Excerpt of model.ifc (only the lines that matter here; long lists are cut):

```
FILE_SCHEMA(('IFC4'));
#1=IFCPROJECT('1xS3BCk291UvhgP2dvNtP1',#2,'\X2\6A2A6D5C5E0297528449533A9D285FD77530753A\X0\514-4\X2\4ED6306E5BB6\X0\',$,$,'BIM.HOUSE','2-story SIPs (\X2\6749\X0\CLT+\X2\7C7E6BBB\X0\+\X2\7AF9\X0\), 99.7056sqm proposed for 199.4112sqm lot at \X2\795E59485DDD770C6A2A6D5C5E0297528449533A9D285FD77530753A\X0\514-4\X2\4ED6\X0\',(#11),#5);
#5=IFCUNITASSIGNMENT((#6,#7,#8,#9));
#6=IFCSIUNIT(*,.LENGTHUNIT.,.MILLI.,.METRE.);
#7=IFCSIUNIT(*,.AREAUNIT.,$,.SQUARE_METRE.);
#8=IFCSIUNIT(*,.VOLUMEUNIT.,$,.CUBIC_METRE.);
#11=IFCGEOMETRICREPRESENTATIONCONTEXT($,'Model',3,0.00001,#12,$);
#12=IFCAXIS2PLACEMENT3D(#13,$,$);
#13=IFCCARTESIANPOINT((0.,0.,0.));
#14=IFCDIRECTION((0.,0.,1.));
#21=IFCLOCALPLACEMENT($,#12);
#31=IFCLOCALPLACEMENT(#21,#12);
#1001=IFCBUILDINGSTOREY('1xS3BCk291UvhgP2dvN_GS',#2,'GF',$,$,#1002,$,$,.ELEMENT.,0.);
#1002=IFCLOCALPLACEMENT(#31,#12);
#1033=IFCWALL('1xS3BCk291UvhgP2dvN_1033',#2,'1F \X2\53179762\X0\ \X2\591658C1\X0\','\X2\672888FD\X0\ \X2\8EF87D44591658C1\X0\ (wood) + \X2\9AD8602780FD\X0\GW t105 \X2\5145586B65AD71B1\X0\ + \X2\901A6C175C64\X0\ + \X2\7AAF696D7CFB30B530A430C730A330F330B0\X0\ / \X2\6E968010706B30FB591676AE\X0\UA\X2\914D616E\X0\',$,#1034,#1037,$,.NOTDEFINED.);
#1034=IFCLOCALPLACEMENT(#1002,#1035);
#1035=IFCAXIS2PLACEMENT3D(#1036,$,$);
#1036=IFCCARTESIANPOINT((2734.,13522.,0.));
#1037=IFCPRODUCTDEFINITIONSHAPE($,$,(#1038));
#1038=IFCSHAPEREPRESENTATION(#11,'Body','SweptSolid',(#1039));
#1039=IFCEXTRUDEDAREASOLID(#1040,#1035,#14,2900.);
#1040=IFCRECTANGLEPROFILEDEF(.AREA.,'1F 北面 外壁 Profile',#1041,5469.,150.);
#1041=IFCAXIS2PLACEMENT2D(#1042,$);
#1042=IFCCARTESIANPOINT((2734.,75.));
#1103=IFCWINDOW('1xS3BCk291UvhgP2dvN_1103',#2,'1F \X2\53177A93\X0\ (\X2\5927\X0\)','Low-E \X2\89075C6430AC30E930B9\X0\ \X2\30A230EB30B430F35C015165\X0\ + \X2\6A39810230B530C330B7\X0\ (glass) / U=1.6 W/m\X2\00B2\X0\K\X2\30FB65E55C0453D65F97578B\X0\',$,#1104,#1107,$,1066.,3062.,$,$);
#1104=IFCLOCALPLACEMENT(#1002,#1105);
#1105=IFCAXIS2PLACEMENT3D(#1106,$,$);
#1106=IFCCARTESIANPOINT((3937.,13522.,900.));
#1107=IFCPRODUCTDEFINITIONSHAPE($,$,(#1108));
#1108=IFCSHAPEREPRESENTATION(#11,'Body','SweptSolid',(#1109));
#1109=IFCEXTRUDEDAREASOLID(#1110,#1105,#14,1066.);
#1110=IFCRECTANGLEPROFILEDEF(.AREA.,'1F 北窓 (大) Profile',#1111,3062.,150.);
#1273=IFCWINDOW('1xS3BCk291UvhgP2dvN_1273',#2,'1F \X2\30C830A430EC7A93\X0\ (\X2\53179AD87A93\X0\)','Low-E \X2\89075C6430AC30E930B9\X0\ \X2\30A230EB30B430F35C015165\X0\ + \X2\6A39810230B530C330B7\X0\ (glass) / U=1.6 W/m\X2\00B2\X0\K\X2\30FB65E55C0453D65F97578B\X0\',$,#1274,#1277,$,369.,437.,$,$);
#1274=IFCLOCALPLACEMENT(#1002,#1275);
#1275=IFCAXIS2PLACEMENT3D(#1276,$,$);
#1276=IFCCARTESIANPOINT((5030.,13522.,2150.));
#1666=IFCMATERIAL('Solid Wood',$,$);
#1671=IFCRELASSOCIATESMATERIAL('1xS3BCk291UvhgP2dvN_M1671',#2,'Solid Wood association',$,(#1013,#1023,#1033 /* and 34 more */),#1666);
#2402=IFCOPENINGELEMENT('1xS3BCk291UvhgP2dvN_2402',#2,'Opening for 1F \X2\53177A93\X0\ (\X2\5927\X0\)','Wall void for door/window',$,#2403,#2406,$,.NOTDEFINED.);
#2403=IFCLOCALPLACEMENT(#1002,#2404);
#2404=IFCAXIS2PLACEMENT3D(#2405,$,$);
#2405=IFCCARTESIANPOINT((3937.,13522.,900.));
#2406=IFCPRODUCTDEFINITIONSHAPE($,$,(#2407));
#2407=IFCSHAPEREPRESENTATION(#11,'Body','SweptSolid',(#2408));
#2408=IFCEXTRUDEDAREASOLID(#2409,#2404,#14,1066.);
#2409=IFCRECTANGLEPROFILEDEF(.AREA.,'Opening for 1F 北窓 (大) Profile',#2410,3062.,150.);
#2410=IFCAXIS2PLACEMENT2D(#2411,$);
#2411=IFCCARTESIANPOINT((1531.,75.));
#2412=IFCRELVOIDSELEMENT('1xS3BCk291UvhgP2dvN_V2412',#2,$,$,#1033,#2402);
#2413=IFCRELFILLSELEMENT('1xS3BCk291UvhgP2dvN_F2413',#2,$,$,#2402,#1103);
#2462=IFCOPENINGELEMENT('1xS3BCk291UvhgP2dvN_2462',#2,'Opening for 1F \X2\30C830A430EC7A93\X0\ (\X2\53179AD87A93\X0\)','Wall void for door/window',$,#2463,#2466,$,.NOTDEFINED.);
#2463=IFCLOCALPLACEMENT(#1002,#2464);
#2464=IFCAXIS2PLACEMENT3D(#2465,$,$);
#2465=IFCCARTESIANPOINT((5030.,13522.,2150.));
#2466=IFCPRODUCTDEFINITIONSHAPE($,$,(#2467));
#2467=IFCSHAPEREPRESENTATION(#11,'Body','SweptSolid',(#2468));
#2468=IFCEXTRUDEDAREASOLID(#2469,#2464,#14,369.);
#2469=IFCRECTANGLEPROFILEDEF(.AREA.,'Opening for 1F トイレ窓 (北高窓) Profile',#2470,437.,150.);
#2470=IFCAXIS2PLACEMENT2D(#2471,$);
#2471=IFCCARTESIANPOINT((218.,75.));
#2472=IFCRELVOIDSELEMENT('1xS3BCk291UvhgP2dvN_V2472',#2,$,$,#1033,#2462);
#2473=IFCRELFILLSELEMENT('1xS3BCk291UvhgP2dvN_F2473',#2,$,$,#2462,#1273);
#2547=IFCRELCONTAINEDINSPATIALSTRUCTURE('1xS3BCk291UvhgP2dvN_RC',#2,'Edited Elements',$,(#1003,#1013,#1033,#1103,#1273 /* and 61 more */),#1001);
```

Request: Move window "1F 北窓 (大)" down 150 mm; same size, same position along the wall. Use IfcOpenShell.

```python
import numpy as np
import ifcopenshell
import ifcopenshell.api.geometry
import ifcopenshell.util.placement
import ifcopenshell.util.unit

model = ifcopenshell.open("model.ifc")
unit_scale = ifcopenshell.util.unit.calculate_unit_scale(model)

window = model.by_guid("1xS3BCk291UvhgP2dvN_1103")
opening = window.FillsVoids[0].RelatingOpeningElement
dz = -0.15 / unit_scale

shift = np.array([0.0, 0.0, dz])
# The window is not placed relative to its opening, so move both.
for product in (opening, window):
    matrix = ifcopenshell.util.placement.get_local_placement(product.ObjectPlacement)
    matrix[:3, 3] += shift
    ifcopenshell.api.geometry.edit_object_placement(model, product=product, matrix=matrix, is_si=False)

print(f"moved by {dz * unit_scale:+.3f} m")

model.write("model_updated.ifc")
```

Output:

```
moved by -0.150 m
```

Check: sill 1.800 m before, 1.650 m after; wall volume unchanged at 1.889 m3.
